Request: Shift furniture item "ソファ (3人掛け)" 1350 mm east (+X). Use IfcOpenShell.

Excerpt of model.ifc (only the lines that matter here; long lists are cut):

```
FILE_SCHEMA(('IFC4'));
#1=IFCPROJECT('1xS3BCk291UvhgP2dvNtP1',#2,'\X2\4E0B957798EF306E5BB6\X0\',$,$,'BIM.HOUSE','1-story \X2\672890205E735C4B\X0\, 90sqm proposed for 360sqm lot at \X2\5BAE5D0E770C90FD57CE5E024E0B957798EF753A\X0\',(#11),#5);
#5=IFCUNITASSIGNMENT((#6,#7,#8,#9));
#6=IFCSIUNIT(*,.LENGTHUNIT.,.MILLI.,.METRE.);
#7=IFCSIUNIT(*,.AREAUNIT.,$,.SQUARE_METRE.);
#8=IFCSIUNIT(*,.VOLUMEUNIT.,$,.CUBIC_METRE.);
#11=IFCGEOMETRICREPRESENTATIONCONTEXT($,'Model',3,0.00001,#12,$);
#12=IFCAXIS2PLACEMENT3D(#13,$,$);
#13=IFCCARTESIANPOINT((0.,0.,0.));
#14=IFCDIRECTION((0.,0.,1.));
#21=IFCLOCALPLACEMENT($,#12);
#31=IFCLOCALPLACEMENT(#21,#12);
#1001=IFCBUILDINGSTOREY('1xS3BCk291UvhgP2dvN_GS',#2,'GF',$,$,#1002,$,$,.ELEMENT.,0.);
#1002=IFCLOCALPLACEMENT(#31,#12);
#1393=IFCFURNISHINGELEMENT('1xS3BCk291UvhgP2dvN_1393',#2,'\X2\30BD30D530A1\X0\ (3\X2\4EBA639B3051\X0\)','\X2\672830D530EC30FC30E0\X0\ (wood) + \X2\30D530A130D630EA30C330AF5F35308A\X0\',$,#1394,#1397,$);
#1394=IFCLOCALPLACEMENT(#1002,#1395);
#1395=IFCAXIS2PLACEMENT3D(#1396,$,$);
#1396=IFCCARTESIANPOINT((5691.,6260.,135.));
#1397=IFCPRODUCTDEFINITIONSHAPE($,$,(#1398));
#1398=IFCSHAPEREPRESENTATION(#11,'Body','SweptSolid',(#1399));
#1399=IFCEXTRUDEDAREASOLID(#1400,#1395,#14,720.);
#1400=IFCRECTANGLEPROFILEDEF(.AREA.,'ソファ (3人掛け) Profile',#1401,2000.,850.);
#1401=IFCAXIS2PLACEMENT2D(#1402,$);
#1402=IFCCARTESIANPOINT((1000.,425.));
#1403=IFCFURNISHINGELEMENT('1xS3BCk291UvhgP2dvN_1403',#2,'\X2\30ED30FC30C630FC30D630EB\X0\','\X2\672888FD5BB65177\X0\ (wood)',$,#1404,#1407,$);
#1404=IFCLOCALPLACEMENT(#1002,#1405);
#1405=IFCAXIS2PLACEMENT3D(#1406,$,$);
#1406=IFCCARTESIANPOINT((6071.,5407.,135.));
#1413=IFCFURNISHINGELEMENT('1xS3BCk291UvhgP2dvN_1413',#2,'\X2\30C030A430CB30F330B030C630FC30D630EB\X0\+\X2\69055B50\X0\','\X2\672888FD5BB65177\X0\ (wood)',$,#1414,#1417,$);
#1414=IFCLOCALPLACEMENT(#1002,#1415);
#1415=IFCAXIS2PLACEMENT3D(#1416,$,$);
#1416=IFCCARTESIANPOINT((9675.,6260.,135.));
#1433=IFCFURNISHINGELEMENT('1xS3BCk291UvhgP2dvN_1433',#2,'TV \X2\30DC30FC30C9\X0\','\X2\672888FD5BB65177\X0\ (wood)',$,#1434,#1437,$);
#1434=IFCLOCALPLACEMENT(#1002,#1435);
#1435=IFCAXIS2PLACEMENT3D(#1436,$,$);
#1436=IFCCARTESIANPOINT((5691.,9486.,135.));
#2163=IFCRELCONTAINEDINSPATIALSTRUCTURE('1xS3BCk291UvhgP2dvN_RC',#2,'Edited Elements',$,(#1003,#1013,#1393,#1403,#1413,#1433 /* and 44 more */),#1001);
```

```python
import ifcopenshell
import ifcopenshell.api.geometry
import ifcopenshell.util.placement

model = ifcopenshell.open("model.ifc")

item = model.by_id(1393)
matrix = ifcopenshell.util.placement.get_local_placement(item.ObjectPlacement)
matrix[0, 3] += 1350.0
ifcopenshell.api.geometry.edit_object_placement(model, product=item, matrix=matrix, is_si=False)

print(ifcopenshell.util.placement.get_local_placement(item.ObjectPlacement).round(3) + 0.0)

model.write("model_edited.ifc")
```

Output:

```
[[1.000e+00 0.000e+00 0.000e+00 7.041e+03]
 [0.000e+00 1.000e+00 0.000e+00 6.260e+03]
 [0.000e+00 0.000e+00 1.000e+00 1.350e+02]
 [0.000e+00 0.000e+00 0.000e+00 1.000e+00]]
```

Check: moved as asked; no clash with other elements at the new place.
